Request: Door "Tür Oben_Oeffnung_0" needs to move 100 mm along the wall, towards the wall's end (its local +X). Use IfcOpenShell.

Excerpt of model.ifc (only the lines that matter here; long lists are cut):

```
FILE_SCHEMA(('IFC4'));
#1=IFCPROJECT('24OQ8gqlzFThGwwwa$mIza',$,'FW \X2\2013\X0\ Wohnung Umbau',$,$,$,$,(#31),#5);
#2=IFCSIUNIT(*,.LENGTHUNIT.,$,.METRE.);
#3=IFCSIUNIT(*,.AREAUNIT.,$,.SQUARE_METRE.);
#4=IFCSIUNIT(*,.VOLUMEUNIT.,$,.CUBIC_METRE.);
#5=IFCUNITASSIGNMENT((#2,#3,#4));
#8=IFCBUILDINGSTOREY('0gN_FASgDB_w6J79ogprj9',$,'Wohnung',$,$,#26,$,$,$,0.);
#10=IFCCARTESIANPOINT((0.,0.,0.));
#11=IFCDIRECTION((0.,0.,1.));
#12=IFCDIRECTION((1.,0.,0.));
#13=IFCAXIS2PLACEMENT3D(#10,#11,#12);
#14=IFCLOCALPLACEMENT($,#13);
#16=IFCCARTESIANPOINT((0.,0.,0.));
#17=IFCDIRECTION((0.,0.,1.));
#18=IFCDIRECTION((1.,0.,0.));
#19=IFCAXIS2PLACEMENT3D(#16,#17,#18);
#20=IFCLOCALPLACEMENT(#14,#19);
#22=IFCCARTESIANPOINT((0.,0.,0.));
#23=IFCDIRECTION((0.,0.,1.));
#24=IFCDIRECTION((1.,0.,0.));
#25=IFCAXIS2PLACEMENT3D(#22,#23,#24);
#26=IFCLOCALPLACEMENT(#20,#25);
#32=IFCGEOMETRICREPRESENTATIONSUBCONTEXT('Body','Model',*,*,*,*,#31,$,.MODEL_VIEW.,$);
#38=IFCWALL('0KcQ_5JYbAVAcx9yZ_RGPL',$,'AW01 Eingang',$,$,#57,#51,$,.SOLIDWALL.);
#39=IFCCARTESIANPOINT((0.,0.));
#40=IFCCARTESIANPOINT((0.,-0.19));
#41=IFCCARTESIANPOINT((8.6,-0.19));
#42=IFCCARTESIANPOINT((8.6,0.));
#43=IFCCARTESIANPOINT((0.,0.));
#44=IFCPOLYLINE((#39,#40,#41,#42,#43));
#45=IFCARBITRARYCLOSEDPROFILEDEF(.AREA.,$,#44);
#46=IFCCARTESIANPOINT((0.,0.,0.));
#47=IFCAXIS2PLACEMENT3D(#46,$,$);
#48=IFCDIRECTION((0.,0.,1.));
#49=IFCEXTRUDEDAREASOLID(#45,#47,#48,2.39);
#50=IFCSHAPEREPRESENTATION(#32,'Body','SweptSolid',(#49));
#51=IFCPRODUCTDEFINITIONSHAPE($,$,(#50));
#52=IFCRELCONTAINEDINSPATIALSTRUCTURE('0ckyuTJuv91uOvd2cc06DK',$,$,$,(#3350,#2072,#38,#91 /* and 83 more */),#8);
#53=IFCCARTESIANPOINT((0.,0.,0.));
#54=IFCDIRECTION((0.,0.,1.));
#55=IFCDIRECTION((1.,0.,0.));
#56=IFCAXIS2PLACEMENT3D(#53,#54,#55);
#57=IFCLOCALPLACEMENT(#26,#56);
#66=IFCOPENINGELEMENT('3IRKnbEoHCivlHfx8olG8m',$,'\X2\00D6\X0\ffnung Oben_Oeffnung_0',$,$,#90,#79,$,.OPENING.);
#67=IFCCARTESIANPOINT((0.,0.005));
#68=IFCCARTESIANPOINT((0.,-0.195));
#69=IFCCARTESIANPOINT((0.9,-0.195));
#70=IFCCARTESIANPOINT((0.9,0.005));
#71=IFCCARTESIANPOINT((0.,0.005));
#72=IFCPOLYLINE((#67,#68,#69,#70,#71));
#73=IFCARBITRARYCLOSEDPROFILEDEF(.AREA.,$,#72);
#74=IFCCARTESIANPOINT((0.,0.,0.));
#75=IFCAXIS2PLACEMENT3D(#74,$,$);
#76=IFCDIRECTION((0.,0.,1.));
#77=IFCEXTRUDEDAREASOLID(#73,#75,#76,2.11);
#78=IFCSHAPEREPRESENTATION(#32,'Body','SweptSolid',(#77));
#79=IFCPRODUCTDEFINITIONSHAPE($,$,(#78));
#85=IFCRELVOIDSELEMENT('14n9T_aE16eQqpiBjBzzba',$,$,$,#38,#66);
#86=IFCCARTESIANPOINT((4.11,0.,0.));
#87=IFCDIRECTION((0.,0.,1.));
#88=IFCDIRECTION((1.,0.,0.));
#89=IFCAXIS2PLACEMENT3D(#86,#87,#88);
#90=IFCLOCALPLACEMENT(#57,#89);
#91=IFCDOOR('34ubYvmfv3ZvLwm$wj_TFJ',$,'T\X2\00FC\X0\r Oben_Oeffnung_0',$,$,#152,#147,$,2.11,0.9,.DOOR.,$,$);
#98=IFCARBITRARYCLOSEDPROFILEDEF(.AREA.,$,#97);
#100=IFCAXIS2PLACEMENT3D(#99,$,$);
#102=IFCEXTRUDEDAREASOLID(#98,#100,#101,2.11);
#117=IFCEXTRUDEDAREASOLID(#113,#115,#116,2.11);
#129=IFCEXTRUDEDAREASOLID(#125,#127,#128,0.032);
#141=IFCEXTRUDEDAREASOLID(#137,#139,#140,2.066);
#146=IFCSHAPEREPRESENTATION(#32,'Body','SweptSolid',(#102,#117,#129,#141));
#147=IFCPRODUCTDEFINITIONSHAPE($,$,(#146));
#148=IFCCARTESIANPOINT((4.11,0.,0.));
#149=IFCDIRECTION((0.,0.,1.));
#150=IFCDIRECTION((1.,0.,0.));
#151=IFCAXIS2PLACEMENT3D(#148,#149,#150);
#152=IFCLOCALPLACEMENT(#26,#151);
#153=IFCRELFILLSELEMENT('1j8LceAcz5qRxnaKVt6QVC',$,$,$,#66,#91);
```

```python
import ifcopenshell
import ifcopenshell.api.geometry
import ifcopenshell.util.placement

model = ifcopenshell.open("model.ifc")

door = model.by_id(91)
opening = door.FillsVoids[0].RelatingOpeningElement
wall = opening.VoidsElements[0].RelatingBuildingElement

wall_matrix = ifcopenshell.util.placement.get_local_placement(wall.ObjectPlacement)
shift = wall_matrix[:3, 0] * 0.1
before = ifcopenshell.util.placement.get_local_placement(door.ObjectPlacement)[:3, 3].copy()

# The door is not placed relative to its opening, so move both.
for product in (opening, door):
    matrix = ifcopenshell.util.placement.get_local_placement(product.ObjectPlacement)
    matrix[:3, 3] += shift
    ifcopenshell.api.geometry.edit_object_placement(model, product=product, matrix=matrix, is_si=False)

after = ifcopenshell.util.placement.get_local_placement(door.ObjectPlacement)[:3, 3]
print("door moved by", (after - before).round(3) + 0.0)

model.write("model_updated.ifc")
```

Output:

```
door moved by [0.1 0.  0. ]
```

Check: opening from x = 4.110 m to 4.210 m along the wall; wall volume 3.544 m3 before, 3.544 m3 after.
